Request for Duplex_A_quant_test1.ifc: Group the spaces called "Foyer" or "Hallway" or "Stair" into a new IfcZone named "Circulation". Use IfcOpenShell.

First a look at what the model holds.

```python
import ifcopenshell

model = ifcopenshell.open("Duplex_A_quant_test1.ifc")
print(model.schema)
seen = {}
for space in model.by_type("IfcSpace"):
    seen[space.LongName] = seen.get(space.LongName, 0) + 1
for name, count in sorted(seen.items(), key=str):
    print(count, "x", name)
print("zones:", [z.Name for z in model.by_type("IfcZone")][:20])
```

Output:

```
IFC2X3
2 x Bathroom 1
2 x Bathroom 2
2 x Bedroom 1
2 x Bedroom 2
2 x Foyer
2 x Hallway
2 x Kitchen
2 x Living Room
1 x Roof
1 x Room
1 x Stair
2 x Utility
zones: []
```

```python
import ifcopenshell
import ifcopenshell.api.group
import ifcopenshell.api.root

model = ifcopenshell.open("Duplex_A_quant_test1.ifc")

names = {"Foyer", "Hallway", "Stair"}
spaces = [s for s in model.by_type("IfcSpace") if s.LongName in names]

zone = ifcopenshell.api.root.create_entity(model, ifc_class="IfcZone", name="Circulation")
ifcopenshell.api.group.assign_group(model, products=spaces, group=zone)
print(len(spaces), "spaces in", zone.Name)

model.write("Duplex_A_quant_test1_updated.ifc")
```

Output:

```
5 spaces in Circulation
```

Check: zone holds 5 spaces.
